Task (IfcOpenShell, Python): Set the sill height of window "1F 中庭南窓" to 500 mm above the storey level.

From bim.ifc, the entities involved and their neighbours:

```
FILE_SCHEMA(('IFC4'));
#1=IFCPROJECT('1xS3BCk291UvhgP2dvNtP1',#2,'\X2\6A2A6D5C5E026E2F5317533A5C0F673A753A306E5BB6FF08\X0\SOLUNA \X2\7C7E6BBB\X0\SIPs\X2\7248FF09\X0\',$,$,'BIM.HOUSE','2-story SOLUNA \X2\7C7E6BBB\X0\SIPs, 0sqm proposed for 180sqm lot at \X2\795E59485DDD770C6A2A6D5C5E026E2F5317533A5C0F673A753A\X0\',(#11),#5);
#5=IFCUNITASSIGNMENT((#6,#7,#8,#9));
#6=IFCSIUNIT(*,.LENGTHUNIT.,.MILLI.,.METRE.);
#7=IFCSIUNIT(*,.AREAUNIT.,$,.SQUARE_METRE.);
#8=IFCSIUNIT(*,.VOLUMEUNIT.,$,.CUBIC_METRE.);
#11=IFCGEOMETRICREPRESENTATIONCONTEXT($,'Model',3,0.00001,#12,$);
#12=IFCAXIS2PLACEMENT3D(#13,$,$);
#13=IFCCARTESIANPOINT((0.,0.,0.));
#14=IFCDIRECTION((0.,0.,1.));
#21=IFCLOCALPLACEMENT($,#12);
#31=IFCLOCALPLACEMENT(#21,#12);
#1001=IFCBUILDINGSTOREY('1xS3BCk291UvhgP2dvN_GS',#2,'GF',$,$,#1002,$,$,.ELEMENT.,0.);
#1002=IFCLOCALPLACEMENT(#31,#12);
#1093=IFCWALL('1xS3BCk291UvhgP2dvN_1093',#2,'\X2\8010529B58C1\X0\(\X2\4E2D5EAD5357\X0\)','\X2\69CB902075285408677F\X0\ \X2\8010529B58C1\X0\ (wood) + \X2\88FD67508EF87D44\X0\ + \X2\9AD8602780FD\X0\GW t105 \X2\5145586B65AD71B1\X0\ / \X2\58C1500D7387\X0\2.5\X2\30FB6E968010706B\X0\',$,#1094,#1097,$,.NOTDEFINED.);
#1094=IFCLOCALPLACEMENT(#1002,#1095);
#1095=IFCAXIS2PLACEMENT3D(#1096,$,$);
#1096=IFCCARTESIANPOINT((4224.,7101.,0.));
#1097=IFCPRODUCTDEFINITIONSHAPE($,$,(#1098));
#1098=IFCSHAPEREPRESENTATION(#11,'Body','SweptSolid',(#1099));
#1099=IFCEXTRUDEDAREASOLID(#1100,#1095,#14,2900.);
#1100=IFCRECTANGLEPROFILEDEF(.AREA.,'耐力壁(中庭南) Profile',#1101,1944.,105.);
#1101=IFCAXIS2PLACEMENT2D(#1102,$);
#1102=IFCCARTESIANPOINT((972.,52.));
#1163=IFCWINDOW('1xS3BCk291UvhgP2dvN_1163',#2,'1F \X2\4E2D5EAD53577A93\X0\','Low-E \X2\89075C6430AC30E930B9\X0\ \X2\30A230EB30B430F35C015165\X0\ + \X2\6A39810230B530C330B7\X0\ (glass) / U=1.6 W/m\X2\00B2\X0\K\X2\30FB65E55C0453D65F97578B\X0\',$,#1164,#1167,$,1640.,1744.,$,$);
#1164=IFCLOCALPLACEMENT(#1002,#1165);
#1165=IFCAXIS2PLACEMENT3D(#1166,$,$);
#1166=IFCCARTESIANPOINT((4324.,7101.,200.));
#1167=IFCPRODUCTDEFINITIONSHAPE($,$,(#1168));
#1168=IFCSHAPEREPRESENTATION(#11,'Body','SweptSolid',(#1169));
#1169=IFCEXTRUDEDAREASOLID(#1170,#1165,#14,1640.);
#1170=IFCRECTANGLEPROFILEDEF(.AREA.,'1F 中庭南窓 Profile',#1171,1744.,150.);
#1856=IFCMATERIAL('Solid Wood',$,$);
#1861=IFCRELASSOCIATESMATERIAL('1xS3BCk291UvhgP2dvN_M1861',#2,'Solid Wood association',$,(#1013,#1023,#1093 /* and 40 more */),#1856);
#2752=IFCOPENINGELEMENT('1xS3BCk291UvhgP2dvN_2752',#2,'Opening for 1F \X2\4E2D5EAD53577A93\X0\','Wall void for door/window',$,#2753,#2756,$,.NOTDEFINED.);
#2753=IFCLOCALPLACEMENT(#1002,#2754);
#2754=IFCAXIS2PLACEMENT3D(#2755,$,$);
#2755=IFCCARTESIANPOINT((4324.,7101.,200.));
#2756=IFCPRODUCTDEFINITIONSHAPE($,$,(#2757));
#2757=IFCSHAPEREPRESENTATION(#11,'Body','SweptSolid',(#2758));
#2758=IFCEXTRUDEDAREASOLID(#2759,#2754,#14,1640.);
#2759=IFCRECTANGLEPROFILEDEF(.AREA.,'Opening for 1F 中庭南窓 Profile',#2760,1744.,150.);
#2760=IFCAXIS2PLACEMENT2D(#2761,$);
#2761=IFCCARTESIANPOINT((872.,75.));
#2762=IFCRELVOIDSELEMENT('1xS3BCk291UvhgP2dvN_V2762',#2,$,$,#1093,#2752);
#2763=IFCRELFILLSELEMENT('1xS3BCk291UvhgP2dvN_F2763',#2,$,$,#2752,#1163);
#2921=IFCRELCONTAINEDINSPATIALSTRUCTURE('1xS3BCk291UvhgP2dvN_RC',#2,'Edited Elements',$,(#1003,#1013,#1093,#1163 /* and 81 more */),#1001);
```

```python
import numpy as np
import ifcopenshell
import ifcopenshell.api.geometry
import ifcopenshell.geom
import ifcopenshell.util.element
import ifcopenshell.util.placement
import ifcopenshell.util.shape
import ifcopenshell.util.unit

model = ifcopenshell.open("bim.ifc")
unit_scale = ifcopenshell.util.unit.calculate_unit_scale(model)

window = model.by_guid("1xS3BCk291UvhgP2dvN_1163")
opening = window.FillsVoids[0].RelatingOpeningElement
storey = ifcopenshell.util.element.get_container(window, ifc_class="IfcBuildingStorey")
level = ifcopenshell.util.placement.get_local_placement(storey.ObjectPlacement)[2, 3]

# The opening's origin need not be at the sill, so measure its lowest point.
shape = ifcopenshell.geom.create_shape(ifcopenshell.geom.settings(), opening)
bottom = ifcopenshell.util.shape.get_shape_bottom_elevation(shape, shape.geometry) / unit_scale
dz = level + 500.0 - bottom

shift = np.array([0.0, 0.0, dz])
# The window is not placed relative to its opening, so move both.
for product in (opening, window):
    matrix = ifcopenshell.util.placement.get_local_placement(product.ObjectPlacement)
    matrix[:3, 3] += shift
    ifcopenshell.api.geometry.edit_object_placement(model, product=product, matrix=matrix, is_si=False)

print(f"moved by {dz * unit_scale:+.3f} m")

model.write("bim-out.ifc")
```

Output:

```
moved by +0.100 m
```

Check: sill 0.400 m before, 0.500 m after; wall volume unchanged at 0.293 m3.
